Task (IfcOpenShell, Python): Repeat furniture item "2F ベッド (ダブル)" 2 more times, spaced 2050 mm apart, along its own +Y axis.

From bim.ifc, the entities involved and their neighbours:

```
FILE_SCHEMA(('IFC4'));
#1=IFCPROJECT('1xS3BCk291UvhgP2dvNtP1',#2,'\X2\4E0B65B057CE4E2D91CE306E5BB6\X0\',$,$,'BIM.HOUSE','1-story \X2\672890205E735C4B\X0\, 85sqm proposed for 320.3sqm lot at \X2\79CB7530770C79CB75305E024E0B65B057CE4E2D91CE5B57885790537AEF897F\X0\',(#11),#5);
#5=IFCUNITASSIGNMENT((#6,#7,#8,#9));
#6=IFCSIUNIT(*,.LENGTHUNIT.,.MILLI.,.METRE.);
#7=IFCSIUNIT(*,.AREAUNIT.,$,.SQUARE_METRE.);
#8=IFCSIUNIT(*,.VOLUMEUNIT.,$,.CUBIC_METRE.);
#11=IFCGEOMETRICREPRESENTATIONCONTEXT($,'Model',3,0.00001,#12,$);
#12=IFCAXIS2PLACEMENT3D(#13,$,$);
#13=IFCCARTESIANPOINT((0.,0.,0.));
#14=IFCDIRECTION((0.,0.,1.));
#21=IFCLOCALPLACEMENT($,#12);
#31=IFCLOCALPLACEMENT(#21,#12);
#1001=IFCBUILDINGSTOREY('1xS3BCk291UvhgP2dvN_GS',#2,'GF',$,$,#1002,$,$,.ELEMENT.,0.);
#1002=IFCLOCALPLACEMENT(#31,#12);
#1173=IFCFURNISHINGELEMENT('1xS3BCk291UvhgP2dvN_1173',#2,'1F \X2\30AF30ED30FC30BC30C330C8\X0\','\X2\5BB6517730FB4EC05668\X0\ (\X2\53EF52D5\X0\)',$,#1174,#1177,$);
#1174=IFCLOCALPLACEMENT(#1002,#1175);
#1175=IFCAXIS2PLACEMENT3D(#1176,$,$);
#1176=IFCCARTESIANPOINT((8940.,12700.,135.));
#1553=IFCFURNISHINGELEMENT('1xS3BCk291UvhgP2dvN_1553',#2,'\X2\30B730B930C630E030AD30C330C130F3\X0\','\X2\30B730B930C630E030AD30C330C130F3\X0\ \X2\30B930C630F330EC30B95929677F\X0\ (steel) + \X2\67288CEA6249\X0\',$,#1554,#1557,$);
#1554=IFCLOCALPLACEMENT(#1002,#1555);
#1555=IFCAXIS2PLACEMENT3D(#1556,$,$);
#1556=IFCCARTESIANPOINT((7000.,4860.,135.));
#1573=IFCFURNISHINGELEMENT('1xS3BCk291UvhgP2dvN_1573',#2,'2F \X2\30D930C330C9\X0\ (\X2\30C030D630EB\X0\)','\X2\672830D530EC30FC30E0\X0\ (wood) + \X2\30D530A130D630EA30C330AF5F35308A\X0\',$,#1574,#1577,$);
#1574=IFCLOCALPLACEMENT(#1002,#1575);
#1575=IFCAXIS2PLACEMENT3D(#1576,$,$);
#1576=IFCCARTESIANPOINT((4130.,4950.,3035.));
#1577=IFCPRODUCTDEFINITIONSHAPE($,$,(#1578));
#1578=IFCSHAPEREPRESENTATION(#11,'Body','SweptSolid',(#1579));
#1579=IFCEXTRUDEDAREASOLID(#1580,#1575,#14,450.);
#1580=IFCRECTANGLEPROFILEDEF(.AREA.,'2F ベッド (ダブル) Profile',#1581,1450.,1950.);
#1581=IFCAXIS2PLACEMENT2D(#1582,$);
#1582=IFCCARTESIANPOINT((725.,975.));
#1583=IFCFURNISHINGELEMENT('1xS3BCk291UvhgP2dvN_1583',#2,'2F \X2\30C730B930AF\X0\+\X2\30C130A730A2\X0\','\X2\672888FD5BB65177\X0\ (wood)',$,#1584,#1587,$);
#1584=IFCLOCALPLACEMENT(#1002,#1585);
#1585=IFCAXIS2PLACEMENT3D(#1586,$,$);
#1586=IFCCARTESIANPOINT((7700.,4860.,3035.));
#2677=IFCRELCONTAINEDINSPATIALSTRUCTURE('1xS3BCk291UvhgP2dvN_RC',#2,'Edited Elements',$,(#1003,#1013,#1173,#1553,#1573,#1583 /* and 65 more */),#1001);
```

```python
import ifcopenshell
import ifcopenshell.api.geometry
import ifcopenshell.api.root
import ifcopenshell.util.element
import ifcopenshell.util.placement
import ifcopenshell.util.unit

model = ifcopenshell.open("bim.ifc")
unit_scale = ifcopenshell.util.unit.calculate_unit_scale(model)


def reuse_history(source, copy):
    """copy_class also copies each property set's owner history, people and application; keep the originals."""
    for rel in copy.IsDefinedBy:
        if rel.is_a("IfcRelDefinesByProperties") and (history := rel.RelatingPropertyDefinition.OwnerHistory):
            rel.RelatingPropertyDefinition.OwnerHistory = source.OwnerHistory
            ifcopenshell.util.element.remove_deep2(model, history)


source = model.by_guid("1xS3BCk291UvhgP2dvN_1573")
base = ifcopenshell.util.placement.get_local_placement(source.ObjectPlacement)
step = base[:3, 1] * 2.05 / unit_scale

for i in range(1, 3):
    copy = ifcopenshell.api.root.copy_class(model, product=source)
    copy.Representation = ifcopenshell.util.element.copy_deep(
        model, source.Representation, exclude=["IfcGeometricRepresentationContext", "IfcRepresentationMap"]
    )
    reuse_history(source, copy)
    matrix = base.copy()
    matrix[:3, 3] += i * step
    print("added at", matrix[:3, 3].round(3) + 0.0)
    ifcopenshell.api.geometry.edit_object_placement(model, product=copy, matrix=matrix, is_si=False)

model.write("bim_updated.ifc")
```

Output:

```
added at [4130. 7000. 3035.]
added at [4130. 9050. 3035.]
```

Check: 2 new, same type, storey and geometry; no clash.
